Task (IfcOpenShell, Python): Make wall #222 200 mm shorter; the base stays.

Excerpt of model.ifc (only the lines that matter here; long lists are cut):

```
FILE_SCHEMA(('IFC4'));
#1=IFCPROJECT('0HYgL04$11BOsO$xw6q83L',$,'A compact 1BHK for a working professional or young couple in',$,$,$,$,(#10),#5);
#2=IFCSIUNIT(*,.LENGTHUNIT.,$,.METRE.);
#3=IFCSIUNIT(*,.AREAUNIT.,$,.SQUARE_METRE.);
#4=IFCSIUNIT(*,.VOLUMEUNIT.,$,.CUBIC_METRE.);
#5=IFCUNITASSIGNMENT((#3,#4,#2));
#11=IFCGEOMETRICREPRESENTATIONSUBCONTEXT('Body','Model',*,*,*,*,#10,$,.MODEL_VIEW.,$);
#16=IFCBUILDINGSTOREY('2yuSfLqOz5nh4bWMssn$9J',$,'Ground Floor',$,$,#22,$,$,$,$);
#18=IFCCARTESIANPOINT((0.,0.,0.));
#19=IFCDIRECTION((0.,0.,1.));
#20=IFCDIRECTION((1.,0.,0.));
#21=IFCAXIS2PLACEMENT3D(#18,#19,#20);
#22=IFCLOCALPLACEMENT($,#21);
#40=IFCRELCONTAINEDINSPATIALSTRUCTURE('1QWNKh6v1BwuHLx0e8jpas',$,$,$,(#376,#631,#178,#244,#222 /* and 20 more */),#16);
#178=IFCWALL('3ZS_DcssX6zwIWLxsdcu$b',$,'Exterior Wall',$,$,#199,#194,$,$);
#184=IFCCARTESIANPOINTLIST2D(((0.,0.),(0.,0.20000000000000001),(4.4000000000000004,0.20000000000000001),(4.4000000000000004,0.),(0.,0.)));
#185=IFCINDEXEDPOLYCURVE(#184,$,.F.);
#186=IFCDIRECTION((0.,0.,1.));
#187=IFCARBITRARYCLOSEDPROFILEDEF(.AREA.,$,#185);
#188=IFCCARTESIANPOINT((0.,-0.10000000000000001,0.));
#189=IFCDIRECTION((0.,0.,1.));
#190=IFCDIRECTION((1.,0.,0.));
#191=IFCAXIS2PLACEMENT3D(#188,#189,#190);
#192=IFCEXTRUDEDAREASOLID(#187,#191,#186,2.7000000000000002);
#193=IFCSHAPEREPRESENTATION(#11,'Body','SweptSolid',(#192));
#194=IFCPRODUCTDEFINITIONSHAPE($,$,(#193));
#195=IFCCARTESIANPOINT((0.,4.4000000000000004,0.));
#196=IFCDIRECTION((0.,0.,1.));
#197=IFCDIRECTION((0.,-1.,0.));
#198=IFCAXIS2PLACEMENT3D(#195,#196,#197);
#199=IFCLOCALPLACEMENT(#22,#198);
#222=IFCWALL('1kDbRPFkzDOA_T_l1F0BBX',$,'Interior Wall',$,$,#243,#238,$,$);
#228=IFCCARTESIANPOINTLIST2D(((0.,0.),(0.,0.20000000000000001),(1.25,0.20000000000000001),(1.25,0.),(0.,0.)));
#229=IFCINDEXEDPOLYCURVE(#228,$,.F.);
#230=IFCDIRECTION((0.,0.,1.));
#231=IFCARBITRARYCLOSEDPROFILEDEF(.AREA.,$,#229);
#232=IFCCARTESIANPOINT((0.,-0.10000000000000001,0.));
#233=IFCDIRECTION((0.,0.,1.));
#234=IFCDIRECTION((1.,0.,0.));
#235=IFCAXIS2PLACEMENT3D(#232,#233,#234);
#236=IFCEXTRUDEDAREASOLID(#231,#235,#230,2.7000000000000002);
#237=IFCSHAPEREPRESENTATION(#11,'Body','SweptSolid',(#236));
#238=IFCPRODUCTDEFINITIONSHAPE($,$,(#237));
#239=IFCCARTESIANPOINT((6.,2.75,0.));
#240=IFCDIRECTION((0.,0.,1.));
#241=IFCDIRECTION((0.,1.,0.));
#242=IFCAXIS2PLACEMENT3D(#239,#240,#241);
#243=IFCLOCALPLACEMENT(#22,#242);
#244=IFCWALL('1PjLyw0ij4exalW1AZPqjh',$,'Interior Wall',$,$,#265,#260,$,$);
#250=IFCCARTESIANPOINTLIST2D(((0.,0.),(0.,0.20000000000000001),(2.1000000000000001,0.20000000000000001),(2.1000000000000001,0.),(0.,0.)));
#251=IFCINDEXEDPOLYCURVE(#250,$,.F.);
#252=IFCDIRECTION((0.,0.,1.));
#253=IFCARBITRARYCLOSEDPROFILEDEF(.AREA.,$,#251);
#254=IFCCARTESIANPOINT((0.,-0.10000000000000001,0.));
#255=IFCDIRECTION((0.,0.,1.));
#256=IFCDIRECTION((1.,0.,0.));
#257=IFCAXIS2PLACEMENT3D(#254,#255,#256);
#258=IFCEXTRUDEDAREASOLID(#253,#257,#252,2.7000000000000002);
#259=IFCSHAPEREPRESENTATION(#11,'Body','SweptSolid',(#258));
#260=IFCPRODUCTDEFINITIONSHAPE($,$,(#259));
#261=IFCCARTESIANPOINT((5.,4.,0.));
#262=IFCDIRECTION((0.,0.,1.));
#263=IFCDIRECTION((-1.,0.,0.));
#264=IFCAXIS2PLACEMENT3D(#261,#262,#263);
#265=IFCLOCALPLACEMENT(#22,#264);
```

```python
import ifcopenshell
import ifcopenshell.geom
import ifcopenshell.util.representation
import ifcopenshell.util.shape

model = ifcopenshell.open("model.ifc")
settings = ifcopenshell.geom.settings()


def volume(element):
    """Net volume in cubic metres, openings subtracted."""
    shape = ifcopenshell.geom.create_shape(settings, element)
    return ifcopenshell.util.shape.get_volume(shape.geometry)


wall = model.by_guid("1kDbRPFkzDOA_T_l1F0BBX")
before = volume(wall)

body = ifcopenshell.util.representation.get_representation(wall, "Model", "Body")
solid = body.Items[0]
old_height = solid.Depth
solid.Depth -= 0.2
after = volume(wall)

print(f"height {old_height:g} -> {solid.Depth:g}, volume {before:.3f} -> {after:.3f} m3")

model.write("model_v2.ifc")
```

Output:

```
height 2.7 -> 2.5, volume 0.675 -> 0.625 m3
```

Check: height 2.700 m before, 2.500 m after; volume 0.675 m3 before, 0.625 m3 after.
